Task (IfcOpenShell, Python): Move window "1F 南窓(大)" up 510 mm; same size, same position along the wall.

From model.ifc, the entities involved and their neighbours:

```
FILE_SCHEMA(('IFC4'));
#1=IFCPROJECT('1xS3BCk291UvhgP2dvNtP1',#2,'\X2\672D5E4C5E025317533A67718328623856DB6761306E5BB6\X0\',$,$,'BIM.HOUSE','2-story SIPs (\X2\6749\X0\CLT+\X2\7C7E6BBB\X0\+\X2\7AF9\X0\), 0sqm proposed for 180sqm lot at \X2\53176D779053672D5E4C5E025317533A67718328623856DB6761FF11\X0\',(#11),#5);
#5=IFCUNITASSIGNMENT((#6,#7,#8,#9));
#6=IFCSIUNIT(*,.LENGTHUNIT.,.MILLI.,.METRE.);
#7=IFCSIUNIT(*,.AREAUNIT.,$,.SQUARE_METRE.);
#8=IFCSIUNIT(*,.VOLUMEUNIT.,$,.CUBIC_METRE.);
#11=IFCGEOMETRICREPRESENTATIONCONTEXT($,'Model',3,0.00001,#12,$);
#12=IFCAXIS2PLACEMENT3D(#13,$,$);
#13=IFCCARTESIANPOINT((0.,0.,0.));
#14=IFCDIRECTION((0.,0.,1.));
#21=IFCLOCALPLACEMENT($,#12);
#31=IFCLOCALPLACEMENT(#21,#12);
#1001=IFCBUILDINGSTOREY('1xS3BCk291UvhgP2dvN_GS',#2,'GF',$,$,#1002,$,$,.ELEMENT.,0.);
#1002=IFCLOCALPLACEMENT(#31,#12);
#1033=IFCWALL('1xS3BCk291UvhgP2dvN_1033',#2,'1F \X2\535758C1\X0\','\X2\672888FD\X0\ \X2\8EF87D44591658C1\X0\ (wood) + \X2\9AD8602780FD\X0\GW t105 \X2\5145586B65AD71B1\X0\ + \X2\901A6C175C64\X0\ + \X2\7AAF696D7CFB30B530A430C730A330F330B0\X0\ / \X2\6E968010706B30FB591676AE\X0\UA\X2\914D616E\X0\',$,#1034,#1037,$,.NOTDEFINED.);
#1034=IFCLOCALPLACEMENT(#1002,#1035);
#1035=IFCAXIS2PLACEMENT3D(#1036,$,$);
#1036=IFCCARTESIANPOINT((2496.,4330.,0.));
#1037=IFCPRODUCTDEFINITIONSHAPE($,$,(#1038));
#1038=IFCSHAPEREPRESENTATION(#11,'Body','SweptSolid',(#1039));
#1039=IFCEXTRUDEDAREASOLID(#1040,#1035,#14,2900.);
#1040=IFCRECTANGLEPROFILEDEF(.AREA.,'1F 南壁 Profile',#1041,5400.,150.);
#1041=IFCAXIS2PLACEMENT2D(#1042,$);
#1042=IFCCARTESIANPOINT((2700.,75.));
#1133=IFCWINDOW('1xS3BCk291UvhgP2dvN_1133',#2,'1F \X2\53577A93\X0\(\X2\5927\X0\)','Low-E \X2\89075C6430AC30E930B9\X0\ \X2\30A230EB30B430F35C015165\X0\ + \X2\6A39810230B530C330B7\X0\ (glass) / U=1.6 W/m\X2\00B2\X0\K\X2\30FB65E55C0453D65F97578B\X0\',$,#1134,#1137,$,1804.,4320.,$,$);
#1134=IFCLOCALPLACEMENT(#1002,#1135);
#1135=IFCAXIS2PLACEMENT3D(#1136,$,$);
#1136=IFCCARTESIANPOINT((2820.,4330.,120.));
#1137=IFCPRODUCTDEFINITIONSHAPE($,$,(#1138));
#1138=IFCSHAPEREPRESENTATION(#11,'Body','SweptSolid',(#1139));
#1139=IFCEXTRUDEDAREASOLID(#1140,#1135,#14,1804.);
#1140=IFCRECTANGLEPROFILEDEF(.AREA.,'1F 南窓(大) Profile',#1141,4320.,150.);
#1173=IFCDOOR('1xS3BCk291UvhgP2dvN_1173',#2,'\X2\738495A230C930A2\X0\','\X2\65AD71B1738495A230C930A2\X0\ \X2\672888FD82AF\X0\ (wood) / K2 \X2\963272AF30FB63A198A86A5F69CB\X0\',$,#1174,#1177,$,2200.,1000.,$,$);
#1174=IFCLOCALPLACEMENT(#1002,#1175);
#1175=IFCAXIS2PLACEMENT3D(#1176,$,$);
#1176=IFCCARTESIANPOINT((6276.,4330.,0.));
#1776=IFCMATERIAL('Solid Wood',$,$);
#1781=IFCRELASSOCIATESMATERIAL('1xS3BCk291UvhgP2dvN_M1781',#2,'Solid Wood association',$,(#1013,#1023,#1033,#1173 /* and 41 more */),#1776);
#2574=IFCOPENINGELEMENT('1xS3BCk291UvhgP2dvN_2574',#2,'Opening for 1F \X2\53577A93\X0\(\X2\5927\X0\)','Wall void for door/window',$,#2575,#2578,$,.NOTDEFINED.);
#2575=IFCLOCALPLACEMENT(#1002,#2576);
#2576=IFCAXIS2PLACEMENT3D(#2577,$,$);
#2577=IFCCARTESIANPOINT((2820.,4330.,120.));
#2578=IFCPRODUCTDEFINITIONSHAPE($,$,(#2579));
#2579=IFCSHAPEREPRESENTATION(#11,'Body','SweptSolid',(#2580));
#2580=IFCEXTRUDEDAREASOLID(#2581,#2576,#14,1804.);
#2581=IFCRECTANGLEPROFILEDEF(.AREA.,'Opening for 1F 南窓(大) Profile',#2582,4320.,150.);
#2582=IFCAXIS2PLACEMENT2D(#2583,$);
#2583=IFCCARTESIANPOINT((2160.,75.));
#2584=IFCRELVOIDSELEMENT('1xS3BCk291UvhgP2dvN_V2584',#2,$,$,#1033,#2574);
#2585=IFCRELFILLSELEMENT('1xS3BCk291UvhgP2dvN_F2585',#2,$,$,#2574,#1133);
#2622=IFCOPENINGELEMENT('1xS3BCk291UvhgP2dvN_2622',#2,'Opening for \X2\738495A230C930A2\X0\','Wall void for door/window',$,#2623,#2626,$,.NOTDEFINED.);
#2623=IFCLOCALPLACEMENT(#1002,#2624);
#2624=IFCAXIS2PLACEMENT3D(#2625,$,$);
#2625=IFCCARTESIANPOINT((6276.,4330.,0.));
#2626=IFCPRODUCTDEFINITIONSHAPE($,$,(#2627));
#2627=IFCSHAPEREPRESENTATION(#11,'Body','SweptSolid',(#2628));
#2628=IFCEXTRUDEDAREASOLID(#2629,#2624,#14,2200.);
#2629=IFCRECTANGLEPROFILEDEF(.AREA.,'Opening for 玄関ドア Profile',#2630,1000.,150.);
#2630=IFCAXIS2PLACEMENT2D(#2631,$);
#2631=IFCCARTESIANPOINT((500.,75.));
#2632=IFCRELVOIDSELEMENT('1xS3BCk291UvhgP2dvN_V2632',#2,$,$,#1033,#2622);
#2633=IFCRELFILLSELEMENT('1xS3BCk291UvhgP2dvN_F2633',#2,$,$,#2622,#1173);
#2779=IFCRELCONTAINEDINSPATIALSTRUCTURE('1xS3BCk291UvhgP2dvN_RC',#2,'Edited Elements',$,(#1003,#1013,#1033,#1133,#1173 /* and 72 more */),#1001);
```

```python
import numpy as np
import ifcopenshell
import ifcopenshell.api.geometry
import ifcopenshell.util.placement
import ifcopenshell.util.unit

model = ifcopenshell.open("model.ifc")
unit_scale = ifcopenshell.util.unit.calculate_unit_scale(model)

window = model.by_id(1133)
opening = window.FillsVoids[0].RelatingOpeningElement
dz = 510.0

shift = np.array([0.0, 0.0, dz])
# The window is not placed relative to its opening, so move both.
for product in (opening, window):
    matrix = ifcopenshell.util.placement.get_local_placement(product.ObjectPlacement)
    matrix[:3, 3] += shift
    ifcopenshell.api.geometry.edit_object_placement(model, product=product, matrix=matrix, is_si=False)

print(f"moved by {dz * unit_scale:+.3f} m")

model.write("model_edited.ifc")
```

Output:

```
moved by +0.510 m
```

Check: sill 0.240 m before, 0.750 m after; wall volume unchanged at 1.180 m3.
